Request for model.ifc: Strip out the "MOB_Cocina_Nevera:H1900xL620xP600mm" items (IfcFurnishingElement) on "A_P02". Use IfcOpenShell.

First a look at what the model holds.

```python
import ifcopenshell
import ifcopenshell.util.element

model = ifcopenshell.open("model.ifc")
print(model.schema)
storey = next(s for s in model.by_type("IfcBuildingStorey") if s.Name == "A_P02")
furniture = [e for e in ifcopenshell.util.element.get_decomposition(storey) if e.is_a("IfcFurnishingElement")]
seen = {}
for e in furniture:
    element_type = ifcopenshell.util.element.get_type(e)
    name = element_type.Name if element_type not in (None, e) else None
    seen[name] = seen.get(name, 0) + 1
for name, count in sorted(seen.items(), key=str):
    print(count, "x", name)
```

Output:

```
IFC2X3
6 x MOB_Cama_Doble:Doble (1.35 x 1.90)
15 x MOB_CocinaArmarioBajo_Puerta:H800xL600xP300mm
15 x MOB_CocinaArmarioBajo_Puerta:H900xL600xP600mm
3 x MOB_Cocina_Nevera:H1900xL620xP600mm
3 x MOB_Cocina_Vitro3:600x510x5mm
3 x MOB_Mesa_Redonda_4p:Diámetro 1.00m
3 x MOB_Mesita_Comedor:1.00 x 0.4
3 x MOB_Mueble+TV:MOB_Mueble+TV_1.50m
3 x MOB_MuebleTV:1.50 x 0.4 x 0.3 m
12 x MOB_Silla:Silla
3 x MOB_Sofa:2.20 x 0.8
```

```python
import ifcopenshell
import ifcopenshell.api.root
import ifcopenshell.util.element

model = ifcopenshell.open("model.ifc")

storey = next(s for s in model.by_type("IfcBuildingStorey") if s.Name == "A_P02")
furniture = [e for e in ifcopenshell.util.element.get_decomposition(storey) if e.is_a("IfcFurnishingElement")]
targets = [e for e in furniture if (t := ifcopenshell.util.element.get_type(e)) not in (None, e) and t.Name == "MOB_Cocina_Nevera:H1900xL620xP600mm"]

for e in targets:
    ifcopenshell.api.root.remove_product(model, product=e)
print(len(targets), "removed")

model.write("model_rev.ifc")
```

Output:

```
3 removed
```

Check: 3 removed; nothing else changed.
